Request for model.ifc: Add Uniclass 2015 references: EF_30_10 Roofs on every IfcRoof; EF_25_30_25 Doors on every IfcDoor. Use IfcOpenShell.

First a look at what the model holds.

```python
import ifcopenshell

model = ifcopenshell.open("model.ifc")
print(model.schema)
print("classifications:", [c.Name for c in model.by_type("IfcClassification")])
for ifc_class in ("IfcDoor", "IfcRoof", "IfcStair", "IfcWall", "IfcWindow"):
    print(ifc_class, len(model.by_type(ifc_class)))
```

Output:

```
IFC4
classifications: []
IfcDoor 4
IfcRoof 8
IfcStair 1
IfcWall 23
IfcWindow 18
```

```python
import ifcopenshell
import ifcopenshell.api.classification

model = ifcopenshell.open("model.ifc")

system = ifcopenshell.api.classification.add_classification(model, classification="Uniclass 2015")

codes = {
    "IfcRoof": ("EF_30_10", "Roofs"),
    "IfcDoor": ("EF_25_30_25", "Doors"),
}
for ifc_class, (code, name) in codes.items():
    products = model.by_type(ifc_class)
    ifcopenshell.api.classification.add_reference(
        model, products=products, classification=system, identification=code, name=name
    )
    print(code, len(products))

model.write("model_edited.ifc")
```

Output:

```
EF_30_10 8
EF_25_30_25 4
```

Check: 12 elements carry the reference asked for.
